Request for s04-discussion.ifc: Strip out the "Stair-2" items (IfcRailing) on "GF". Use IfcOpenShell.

First a look at what the model holds.

```python
import ifcopenshell
import ifcopenshell.util.element

model = ifcopenshell.open("s04-discussion.ifc")
print(model.schema)
storey = next(s for s in model.by_type("IfcBuildingStorey") if s.Name == "GF")
railings = [e for e in ifcopenshell.util.element.get_decomposition(storey) if e.is_a("IfcRailing")]
seen = {}
for e in railings:
    element_type = ifcopenshell.util.element.get_type(e)
    name = element_type.Name if element_type not in (None, e) else None
    seen[name] = seen.get(name, 0) + 1
for name, count in sorted(seen.items(), key=str):
    print(count, "x", name)
```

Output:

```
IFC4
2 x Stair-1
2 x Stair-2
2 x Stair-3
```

```python
import ifcopenshell
import ifcopenshell.api.root
import ifcopenshell.util.element

model = ifcopenshell.open("s04-discussion.ifc")

storey = next(s for s in model.by_type("IfcBuildingStorey") if s.Name == "GF")
railings = [e for e in ifcopenshell.util.element.get_decomposition(storey) if e.is_a("IfcRailing")]
targets = [e for e in railings if (t := ifcopenshell.util.element.get_type(e)) not in (None, e) and t.Name == "Stair-2"]

for e in targets:
    ifcopenshell.api.root.remove_product(model, product=e)
print(len(targets), "removed")

model.write("s04-discussion_rev.ifc")
```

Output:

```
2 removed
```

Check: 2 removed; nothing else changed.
